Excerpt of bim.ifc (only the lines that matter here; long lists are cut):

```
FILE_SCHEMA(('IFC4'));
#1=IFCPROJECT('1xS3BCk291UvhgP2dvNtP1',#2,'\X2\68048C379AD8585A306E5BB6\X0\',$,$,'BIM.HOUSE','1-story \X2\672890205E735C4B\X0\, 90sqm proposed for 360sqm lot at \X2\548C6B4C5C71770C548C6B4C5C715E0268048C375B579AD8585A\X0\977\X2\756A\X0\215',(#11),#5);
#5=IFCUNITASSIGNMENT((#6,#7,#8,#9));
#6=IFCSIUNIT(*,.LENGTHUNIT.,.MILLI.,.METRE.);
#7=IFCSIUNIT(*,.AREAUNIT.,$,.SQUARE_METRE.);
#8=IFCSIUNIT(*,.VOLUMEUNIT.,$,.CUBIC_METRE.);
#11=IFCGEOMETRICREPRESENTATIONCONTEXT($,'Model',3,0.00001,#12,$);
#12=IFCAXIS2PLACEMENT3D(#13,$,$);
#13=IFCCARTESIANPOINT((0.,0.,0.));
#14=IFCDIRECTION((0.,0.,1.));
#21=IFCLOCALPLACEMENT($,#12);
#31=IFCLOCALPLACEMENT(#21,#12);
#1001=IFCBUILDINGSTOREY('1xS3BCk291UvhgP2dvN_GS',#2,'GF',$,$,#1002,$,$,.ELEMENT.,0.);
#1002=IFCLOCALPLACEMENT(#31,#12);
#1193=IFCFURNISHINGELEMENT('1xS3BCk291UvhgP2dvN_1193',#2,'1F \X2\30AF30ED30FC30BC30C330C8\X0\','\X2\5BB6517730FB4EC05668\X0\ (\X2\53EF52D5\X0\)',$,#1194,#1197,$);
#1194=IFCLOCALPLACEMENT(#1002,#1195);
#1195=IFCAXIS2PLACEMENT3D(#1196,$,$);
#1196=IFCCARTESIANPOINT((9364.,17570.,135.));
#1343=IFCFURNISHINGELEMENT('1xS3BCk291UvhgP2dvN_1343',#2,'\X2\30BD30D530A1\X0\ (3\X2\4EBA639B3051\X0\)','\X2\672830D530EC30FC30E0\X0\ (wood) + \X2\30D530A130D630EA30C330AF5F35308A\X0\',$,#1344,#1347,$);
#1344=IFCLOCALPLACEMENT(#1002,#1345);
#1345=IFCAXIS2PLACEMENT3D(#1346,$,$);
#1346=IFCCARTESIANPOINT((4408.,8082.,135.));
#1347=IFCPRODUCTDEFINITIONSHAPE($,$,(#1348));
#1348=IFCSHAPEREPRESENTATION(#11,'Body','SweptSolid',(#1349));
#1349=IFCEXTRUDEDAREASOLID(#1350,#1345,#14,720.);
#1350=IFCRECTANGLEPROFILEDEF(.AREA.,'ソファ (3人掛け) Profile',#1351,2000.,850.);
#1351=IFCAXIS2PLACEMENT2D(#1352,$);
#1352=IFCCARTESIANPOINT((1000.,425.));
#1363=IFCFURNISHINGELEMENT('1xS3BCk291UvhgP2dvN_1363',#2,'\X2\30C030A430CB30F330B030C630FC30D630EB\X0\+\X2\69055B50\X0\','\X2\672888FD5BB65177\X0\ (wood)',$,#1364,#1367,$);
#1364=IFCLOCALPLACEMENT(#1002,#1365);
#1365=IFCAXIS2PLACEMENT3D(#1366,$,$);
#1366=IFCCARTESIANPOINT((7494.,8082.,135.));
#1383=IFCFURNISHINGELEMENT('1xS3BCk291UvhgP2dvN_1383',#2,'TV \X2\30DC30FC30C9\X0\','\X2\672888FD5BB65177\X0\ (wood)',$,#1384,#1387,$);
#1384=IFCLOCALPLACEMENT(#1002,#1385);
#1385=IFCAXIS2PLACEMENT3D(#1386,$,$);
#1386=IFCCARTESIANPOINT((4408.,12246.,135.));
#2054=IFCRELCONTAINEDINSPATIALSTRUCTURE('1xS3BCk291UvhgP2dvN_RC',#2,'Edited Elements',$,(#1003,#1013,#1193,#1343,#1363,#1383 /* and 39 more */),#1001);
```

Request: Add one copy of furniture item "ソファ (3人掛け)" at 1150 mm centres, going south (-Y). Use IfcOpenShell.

```python
import numpy as np
import ifcopenshell
import ifcopenshell.api.geometry
import ifcopenshell.api.root
import ifcopenshell.util.element
import ifcopenshell.util.placement
import ifcopenshell.util.unit

model = ifcopenshell.open("bim.ifc")
unit_scale = ifcopenshell.util.unit.calculate_unit_scale(model)


def reuse_history(source, copy):
    """copy_class also copies each property set's owner history, people and application; keep the originals."""
    for rel in copy.IsDefinedBy:
        if rel.is_a("IfcRelDefinesByProperties") and (history := rel.RelatingPropertyDefinition.OwnerHistory):
            rel.RelatingPropertyDefinition.OwnerHistory = source.OwnerHistory
            ifcopenshell.util.element.remove_deep2(model, history)


source = model.by_guid("1xS3BCk291UvhgP2dvN_1343")
base = ifcopenshell.util.placement.get_local_placement(source.ObjectPlacement)
step = np.array([0.0, -1.0, 0.0]) * 1.15 / unit_scale

for i in range(1, 2):
    copy = ifcopenshell.api.root.copy_class(model, product=source)
    copy.Representation = ifcopenshell.util.element.copy_deep(
        model, source.Representation, exclude=["IfcGeometricRepresentationContext", "IfcRepresentationMap"]
    )
    reuse_history(source, copy)
    matrix = base.copy()
    matrix[:3, 3] += i * step
    print("added at", matrix[:3, 3].round(3) + 0.0)
    ifcopenshell.api.geometry.edit_object_placement(model, product=copy, matrix=matrix, is_si=False)

model.write("bim_rev.ifc")
```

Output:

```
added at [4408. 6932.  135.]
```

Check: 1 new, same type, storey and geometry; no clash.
